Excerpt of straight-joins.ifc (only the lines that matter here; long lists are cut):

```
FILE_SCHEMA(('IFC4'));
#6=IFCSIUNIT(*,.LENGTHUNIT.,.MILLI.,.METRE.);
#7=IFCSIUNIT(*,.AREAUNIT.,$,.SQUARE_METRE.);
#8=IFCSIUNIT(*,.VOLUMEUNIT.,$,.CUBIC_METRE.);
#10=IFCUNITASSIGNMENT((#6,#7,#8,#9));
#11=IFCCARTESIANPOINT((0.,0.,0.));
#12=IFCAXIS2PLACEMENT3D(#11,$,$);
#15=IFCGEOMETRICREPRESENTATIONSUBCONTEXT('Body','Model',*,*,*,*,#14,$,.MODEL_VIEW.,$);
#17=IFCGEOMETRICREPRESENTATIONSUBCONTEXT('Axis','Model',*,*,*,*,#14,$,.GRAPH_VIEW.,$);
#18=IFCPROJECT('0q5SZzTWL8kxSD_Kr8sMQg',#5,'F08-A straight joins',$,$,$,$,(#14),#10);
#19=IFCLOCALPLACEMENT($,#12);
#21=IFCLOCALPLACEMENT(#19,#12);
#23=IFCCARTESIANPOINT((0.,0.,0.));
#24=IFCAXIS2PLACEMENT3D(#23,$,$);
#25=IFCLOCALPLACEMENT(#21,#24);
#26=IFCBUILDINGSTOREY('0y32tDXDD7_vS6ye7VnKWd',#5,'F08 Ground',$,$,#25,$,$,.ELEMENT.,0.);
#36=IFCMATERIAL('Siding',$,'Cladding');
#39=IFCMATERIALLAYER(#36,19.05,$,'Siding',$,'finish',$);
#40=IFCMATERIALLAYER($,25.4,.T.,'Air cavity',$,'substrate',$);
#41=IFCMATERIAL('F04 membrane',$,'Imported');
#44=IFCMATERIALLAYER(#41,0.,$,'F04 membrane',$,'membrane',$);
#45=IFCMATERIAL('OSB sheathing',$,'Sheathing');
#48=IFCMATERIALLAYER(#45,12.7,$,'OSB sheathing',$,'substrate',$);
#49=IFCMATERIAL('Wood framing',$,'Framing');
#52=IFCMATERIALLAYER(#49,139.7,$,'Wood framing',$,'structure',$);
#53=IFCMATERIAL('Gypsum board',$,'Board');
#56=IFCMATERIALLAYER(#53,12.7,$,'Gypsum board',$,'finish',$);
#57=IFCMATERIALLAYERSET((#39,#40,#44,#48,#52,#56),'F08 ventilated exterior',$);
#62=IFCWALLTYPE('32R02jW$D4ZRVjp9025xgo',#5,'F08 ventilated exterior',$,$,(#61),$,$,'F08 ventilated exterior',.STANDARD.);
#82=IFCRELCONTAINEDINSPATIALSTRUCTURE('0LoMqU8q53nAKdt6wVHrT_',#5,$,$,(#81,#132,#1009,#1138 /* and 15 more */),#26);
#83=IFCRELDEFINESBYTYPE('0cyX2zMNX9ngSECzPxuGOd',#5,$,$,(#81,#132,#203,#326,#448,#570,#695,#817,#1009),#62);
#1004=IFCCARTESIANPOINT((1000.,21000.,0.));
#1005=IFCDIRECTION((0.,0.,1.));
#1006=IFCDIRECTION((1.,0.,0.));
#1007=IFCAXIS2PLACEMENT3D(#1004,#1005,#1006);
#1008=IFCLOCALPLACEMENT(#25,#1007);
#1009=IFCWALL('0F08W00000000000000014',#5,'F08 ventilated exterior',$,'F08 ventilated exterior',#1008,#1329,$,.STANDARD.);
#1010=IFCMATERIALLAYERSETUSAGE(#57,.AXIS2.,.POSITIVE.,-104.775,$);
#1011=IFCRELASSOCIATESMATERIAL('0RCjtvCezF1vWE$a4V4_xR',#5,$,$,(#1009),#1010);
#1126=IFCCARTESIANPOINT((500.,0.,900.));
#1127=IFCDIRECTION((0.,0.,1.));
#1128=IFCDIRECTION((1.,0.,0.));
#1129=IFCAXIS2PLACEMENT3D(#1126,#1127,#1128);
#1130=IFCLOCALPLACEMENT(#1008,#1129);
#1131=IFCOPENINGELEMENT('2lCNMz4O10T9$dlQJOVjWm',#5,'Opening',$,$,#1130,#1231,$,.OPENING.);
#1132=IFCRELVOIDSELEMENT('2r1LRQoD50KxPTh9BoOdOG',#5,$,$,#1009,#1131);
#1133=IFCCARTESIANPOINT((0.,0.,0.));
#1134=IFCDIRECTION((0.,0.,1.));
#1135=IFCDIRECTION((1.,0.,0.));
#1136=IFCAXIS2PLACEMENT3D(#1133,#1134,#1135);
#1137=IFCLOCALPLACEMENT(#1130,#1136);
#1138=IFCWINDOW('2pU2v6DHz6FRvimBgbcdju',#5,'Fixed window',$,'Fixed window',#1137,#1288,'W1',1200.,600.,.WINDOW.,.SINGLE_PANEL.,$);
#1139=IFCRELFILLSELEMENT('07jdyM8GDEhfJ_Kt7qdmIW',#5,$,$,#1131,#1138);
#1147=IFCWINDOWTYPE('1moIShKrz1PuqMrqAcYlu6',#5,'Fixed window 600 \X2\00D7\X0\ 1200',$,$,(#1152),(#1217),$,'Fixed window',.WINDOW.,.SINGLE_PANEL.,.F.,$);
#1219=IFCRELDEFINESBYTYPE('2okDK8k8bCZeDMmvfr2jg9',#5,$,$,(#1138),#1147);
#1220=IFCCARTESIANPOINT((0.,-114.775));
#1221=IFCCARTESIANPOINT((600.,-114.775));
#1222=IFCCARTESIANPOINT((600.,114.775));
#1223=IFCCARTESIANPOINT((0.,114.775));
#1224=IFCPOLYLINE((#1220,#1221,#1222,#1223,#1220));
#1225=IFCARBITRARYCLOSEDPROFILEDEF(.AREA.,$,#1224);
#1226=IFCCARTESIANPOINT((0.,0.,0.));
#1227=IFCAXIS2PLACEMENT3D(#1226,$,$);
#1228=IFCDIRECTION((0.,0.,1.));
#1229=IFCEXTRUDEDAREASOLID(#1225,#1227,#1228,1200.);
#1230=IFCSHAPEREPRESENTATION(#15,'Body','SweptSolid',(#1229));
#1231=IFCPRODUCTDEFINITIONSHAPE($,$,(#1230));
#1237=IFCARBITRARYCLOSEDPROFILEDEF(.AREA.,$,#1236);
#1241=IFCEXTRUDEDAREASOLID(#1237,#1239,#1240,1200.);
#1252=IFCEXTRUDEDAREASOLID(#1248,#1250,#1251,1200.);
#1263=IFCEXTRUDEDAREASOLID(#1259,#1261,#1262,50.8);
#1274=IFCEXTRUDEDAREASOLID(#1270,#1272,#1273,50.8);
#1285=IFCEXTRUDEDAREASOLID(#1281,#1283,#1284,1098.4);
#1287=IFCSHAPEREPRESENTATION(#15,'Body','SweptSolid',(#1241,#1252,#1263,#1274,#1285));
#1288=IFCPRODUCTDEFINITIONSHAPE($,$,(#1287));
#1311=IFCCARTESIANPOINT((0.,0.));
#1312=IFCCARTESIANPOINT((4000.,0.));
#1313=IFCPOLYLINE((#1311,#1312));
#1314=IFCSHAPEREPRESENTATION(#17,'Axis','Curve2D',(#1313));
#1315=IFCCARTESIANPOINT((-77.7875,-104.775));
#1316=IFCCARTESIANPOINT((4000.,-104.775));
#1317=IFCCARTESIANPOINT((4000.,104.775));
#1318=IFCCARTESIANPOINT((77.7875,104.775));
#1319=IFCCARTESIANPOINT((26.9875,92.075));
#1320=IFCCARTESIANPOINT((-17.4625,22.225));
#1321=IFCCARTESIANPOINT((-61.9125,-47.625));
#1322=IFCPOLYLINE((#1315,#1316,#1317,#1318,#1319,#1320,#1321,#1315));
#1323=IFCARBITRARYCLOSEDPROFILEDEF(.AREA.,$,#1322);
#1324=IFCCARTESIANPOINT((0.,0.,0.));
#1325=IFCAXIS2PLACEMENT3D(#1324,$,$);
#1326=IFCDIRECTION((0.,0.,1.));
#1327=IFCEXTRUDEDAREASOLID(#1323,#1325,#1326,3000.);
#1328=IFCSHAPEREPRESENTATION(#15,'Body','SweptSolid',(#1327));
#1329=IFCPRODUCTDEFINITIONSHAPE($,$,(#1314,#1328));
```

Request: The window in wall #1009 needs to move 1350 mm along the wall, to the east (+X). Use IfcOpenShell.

```python
import ifcopenshell
import ifcopenshell.api.geometry
import ifcopenshell.util.placement

model = ifcopenshell.open("straight-joins.ifc")

window = model.by_id(1138)
opening = window.FillsVoids[0].RelatingOpeningElement
wall = opening.VoidsElements[0].RelatingBuildingElement

wall_matrix = ifcopenshell.util.placement.get_local_placement(wall.ObjectPlacement)
shift = wall_matrix[:3, 0] * 1350.0
before = ifcopenshell.util.placement.get_local_placement(window.ObjectPlacement)[:3, 3].copy()

# The window is placed relative to its opening, so it follows when the opening moves.
matrix = ifcopenshell.util.placement.get_local_placement(opening.ObjectPlacement)
matrix[:3, 3] += shift
ifcopenshell.api.geometry.edit_object_placement(
    model, product=opening, matrix=matrix, is_si=False, should_transform_children=True
)

after = ifcopenshell.util.placement.get_local_placement(window.ObjectPlacement)[:3, 3]
print("window moved by", (after - before).round(3) + 0.0)

model.write("straight-joins-out.ifc")
```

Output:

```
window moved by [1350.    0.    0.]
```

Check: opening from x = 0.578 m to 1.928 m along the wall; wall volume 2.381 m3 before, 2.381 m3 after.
